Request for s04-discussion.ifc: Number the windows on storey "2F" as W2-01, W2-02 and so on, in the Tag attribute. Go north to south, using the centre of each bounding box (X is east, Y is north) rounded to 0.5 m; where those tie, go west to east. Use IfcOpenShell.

First a look at what the model holds.

```python
import ifcopenshell
import ifcopenshell.util.element
import ifcopenshell.util.placement

model = ifcopenshell.open("s04-discussion.ifc")
print(model.schema)
storey = next(s for s in model.by_type("IfcBuildingStorey") if s.Name == "2F")
windows = [e for e in ifcopenshell.util.element.get_decomposition(storey) if e.is_a("IfcWindow")]
for e in sorted(windows, key=lambda e: e.id()):
    origin = ifcopenshell.util.placement.get_local_placement(e.ObjectPlacement)[:3, 3]
    print(e.id(), e.Tag, e.Name, origin.round(2) + 0.0, sep=" | ")
```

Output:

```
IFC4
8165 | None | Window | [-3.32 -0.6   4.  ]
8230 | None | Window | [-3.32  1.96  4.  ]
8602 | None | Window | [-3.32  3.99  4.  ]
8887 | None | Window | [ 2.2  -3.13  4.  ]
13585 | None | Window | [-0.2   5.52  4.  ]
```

```python
import ifcopenshell
import ifcopenshell.geom
import ifcopenshell.util.element
import ifcopenshell.util.shape

model = ifcopenshell.open("s04-discussion.ifc")
settings = ifcopenshell.geom.settings()
settings.set("use-world-coords", True)


def centre(element):
    shape = ifcopenshell.geom.create_shape(settings, element)
    return ifcopenshell.util.shape.get_bbox_centroid(shape.geometry)


storey = next(s for s in model.by_type("IfcBuildingStorey") if s.Name == "2F")
windows = [e for e in ifcopenshell.util.element.get_decomposition(storey) if e.is_a("IfcWindow")]

# Insertion points can sit at a corner or the storey origin, so sort by the geometry (in metres).
centres = {e: centre(e) for e in windows}
windows.sort(key=lambda e: (-round(centres[e][1] / 0.5), centres[e][0]))

for i, e in enumerate(windows, start=1):
    number = f"W2-{i:02d}"
    e.Tag = number
    print(e.id(), number)

model.write("s04-discussion_updated.ifc")
```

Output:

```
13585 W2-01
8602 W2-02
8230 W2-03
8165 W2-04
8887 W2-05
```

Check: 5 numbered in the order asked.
